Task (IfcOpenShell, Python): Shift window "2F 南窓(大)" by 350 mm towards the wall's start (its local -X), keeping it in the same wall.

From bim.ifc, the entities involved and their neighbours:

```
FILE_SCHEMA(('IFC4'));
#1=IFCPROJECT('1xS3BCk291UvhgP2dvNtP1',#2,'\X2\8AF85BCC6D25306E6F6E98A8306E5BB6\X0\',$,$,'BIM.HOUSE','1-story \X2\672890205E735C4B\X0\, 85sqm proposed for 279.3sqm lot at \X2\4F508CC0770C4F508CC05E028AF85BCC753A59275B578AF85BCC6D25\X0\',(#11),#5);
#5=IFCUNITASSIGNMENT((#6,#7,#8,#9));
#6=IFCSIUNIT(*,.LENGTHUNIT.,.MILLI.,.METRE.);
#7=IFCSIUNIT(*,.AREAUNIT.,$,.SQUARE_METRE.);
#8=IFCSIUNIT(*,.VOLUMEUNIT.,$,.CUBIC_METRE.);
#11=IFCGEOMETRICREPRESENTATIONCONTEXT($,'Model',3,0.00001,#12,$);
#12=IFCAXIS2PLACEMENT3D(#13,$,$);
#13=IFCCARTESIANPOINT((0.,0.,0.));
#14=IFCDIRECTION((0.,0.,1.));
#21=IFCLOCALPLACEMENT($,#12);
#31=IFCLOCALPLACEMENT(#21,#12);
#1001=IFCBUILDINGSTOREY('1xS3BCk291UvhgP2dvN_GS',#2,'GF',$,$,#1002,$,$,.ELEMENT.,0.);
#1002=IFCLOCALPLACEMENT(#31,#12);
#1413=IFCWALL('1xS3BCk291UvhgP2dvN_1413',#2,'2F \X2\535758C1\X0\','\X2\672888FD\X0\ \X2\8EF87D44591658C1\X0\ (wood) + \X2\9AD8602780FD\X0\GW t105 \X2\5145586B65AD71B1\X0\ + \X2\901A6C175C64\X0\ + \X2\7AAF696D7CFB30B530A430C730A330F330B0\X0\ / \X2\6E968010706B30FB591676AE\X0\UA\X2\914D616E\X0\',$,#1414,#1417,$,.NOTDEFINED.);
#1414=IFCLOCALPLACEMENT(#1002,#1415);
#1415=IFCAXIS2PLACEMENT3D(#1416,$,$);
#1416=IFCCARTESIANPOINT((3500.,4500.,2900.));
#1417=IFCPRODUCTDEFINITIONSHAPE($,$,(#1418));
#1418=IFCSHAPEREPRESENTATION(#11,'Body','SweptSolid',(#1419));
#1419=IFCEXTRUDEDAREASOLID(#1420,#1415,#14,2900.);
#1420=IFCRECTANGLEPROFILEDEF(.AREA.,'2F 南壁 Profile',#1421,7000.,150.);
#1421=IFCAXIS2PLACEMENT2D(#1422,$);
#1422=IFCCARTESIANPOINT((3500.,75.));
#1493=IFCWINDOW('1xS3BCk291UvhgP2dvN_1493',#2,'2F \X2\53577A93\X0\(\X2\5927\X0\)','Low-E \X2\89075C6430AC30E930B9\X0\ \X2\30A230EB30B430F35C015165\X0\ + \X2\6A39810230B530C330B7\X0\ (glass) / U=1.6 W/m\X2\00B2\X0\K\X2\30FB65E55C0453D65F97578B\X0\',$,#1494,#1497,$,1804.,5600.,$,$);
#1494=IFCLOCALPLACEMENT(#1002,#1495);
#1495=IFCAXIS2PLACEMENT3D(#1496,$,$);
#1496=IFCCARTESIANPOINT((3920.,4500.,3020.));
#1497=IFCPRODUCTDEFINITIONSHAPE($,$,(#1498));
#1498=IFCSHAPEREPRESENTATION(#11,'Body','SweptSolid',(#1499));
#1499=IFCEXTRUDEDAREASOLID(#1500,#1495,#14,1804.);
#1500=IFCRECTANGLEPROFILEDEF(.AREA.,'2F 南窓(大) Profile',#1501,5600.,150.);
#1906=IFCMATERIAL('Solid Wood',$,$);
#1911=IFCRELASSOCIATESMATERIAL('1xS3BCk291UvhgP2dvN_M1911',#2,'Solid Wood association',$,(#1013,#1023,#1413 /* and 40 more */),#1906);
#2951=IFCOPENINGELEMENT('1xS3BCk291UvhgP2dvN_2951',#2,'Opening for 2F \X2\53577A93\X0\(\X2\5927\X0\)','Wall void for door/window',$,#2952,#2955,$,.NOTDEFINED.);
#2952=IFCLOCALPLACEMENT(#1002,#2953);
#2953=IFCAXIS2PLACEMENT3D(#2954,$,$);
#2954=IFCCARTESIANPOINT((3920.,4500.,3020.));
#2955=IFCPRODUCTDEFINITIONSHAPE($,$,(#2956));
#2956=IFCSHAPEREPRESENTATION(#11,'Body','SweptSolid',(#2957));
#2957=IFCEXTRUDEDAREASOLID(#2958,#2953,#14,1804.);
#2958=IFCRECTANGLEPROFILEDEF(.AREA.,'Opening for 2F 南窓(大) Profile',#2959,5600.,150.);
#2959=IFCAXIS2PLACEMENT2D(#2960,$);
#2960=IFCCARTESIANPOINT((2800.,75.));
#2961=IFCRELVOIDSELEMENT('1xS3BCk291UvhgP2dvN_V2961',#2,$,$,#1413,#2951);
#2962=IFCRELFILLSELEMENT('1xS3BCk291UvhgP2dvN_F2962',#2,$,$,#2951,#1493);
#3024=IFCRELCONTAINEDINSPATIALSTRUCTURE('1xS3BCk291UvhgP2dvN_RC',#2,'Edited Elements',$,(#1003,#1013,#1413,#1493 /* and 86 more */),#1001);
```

```python
import ifcopenshell
import ifcopenshell.api.geometry
import ifcopenshell.util.placement
import ifcopenshell.util.unit

model = ifcopenshell.open("bim.ifc")
unit_scale = ifcopenshell.util.unit.calculate_unit_scale(model)

window = model.by_guid("1xS3BCk291UvhgP2dvN_1493")
opening = window.FillsVoids[0].RelatingOpeningElement
wall = opening.VoidsElements[0].RelatingBuildingElement

wall_matrix = ifcopenshell.util.placement.get_local_placement(wall.ObjectPlacement)
shift = wall_matrix[:3, 0] * -0.35 / unit_scale
before = ifcopenshell.util.placement.get_local_placement(window.ObjectPlacement)[:3, 3].copy()

# The window is not placed relative to its opening, so move both.
for product in (opening, window):
    matrix = ifcopenshell.util.placement.get_local_placement(product.ObjectPlacement)
    matrix[:3, 3] += shift
    ifcopenshell.api.geometry.edit_object_placement(model, product=product, matrix=matrix, is_si=False)

after = ifcopenshell.util.placement.get_local_placement(window.ObjectPlacement)[:3, 3]
print("window moved by", (after - before).round(3) + 0.0)

model.write("bim-out.ifc")
```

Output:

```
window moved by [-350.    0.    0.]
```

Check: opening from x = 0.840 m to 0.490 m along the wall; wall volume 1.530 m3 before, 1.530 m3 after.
